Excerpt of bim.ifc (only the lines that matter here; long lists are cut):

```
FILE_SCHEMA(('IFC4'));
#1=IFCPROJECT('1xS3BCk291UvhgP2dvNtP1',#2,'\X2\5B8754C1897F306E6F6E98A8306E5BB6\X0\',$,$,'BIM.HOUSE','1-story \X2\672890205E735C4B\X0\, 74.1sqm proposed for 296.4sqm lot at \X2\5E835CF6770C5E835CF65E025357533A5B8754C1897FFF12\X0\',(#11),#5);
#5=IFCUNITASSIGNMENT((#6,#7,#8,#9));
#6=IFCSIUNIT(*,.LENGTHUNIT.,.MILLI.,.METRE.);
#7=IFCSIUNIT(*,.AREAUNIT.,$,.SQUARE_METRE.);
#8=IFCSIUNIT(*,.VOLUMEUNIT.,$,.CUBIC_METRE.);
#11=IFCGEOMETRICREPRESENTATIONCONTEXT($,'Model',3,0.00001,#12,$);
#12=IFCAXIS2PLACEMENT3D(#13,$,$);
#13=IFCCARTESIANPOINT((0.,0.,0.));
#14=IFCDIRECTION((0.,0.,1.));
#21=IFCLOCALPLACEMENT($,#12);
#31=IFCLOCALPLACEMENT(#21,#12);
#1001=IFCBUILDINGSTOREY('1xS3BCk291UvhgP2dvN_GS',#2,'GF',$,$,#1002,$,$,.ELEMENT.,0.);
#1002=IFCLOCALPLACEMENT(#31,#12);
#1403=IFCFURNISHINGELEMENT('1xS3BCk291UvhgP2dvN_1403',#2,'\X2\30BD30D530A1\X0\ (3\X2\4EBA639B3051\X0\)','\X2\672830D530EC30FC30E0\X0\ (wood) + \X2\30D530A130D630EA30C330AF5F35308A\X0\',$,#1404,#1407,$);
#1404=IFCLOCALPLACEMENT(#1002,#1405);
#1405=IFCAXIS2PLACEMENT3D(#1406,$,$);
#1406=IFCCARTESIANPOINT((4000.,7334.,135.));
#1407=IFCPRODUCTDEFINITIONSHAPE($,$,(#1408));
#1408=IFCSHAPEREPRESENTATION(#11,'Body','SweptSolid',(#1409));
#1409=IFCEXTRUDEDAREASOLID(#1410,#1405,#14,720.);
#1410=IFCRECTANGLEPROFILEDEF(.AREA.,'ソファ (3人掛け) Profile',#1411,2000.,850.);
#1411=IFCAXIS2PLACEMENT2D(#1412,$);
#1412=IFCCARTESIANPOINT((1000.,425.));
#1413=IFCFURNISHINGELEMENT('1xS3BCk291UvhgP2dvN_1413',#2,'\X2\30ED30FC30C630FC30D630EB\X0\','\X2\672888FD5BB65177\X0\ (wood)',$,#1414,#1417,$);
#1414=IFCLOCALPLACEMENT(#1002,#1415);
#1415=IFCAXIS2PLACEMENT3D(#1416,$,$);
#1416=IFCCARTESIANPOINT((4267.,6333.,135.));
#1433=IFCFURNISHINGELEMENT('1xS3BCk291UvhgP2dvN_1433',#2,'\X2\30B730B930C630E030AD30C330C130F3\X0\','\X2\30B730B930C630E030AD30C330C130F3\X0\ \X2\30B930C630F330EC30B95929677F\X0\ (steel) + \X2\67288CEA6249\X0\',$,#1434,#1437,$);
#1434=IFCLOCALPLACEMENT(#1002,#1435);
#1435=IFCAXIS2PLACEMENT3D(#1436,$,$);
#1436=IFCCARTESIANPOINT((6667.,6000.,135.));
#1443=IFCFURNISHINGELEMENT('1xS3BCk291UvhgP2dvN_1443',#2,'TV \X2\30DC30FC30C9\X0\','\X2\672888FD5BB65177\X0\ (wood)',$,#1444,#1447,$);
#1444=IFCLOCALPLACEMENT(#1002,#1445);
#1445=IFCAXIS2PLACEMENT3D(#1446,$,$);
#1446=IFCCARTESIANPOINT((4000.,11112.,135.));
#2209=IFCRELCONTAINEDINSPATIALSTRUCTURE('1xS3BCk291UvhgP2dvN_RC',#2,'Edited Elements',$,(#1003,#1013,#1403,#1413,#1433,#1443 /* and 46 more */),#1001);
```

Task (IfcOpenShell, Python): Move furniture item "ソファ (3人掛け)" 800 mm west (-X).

```python
import ifcopenshell
import ifcopenshell.api.geometry
import ifcopenshell.util.placement
import ifcopenshell.util.unit

model = ifcopenshell.open("bim.ifc")
unit_scale = ifcopenshell.util.unit.calculate_unit_scale(model)

item = model.by_guid("1xS3BCk291UvhgP2dvN_1403")
matrix = ifcopenshell.util.placement.get_local_placement(item.ObjectPlacement)
matrix[0, 3] -= 0.8 / unit_scale
ifcopenshell.api.geometry.edit_object_placement(model, product=item, matrix=matrix, is_si=False)

print(ifcopenshell.util.placement.get_local_placement(item.ObjectPlacement).round(3) + 0.0)

model.write("bim_updated.ifc")
```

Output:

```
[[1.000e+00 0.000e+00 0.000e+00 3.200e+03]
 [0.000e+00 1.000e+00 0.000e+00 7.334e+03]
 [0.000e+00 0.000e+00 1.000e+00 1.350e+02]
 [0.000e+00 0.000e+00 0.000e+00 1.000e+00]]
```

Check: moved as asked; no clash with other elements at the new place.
